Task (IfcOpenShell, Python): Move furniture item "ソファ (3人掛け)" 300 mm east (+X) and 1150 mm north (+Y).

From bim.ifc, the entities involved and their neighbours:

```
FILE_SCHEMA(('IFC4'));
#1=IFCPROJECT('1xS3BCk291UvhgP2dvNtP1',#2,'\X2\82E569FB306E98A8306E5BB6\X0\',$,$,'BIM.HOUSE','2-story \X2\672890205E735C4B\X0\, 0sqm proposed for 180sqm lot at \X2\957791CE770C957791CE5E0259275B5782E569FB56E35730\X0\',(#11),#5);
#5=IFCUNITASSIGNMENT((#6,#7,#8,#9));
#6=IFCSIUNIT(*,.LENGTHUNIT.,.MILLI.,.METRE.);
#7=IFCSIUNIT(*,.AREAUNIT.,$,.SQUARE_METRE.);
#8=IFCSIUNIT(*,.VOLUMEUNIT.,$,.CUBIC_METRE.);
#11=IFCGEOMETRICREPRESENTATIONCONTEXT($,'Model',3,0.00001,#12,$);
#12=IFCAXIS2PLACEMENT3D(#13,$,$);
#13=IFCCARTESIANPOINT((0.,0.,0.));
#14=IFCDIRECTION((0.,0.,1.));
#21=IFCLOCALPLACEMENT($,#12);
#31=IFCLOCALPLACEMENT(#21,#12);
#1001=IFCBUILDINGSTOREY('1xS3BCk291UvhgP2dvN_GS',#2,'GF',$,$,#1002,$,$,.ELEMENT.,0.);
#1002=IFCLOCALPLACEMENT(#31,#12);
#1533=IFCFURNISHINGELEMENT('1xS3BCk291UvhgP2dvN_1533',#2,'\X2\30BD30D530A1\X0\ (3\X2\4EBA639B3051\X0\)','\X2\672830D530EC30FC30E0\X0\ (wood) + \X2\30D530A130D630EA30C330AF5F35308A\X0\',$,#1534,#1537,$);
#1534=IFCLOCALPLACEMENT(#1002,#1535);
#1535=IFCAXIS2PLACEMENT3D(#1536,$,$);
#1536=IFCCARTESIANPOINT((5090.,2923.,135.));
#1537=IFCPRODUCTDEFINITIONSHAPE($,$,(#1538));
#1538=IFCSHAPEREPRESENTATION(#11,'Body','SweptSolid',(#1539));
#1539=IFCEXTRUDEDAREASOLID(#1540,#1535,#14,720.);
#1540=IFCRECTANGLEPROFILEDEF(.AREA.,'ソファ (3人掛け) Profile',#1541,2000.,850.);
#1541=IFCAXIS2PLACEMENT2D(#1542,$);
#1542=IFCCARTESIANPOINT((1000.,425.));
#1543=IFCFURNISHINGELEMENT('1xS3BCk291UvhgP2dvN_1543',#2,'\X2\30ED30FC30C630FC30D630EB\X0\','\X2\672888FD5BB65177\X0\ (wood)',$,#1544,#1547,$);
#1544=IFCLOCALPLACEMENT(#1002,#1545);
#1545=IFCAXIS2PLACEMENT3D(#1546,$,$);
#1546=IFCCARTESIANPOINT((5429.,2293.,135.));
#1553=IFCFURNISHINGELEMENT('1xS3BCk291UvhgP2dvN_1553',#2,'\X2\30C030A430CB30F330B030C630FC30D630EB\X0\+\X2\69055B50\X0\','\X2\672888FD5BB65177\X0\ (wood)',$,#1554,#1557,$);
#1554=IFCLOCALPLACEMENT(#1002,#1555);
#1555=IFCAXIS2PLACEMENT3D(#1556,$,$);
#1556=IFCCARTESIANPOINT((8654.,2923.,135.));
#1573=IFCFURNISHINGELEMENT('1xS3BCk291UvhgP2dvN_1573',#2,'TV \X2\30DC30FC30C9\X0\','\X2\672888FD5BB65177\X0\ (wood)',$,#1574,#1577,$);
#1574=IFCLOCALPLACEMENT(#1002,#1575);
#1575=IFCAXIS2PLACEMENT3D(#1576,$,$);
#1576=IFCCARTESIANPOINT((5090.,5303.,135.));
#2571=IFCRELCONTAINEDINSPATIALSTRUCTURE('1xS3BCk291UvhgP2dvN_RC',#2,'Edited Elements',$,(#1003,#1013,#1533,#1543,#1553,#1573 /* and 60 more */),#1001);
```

```python
import ifcopenshell
import ifcopenshell.api.geometry
import ifcopenshell.util.placement

model = ifcopenshell.open("bim.ifc")

item = model.by_id(1533)
matrix = ifcopenshell.util.placement.get_local_placement(item.ObjectPlacement)
matrix[0, 3] += 300.0
matrix[1, 3] += 1150.0
ifcopenshell.api.geometry.edit_object_placement(model, product=item, matrix=matrix, is_si=False)

print(ifcopenshell.util.placement.get_local_placement(item.ObjectPlacement).round(3) + 0.0)

model.write("bim_v2.ifc")
```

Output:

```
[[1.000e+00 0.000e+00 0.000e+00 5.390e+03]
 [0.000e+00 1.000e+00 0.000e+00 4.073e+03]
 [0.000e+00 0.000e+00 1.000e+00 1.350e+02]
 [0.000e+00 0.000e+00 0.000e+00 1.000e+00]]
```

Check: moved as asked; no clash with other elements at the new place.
